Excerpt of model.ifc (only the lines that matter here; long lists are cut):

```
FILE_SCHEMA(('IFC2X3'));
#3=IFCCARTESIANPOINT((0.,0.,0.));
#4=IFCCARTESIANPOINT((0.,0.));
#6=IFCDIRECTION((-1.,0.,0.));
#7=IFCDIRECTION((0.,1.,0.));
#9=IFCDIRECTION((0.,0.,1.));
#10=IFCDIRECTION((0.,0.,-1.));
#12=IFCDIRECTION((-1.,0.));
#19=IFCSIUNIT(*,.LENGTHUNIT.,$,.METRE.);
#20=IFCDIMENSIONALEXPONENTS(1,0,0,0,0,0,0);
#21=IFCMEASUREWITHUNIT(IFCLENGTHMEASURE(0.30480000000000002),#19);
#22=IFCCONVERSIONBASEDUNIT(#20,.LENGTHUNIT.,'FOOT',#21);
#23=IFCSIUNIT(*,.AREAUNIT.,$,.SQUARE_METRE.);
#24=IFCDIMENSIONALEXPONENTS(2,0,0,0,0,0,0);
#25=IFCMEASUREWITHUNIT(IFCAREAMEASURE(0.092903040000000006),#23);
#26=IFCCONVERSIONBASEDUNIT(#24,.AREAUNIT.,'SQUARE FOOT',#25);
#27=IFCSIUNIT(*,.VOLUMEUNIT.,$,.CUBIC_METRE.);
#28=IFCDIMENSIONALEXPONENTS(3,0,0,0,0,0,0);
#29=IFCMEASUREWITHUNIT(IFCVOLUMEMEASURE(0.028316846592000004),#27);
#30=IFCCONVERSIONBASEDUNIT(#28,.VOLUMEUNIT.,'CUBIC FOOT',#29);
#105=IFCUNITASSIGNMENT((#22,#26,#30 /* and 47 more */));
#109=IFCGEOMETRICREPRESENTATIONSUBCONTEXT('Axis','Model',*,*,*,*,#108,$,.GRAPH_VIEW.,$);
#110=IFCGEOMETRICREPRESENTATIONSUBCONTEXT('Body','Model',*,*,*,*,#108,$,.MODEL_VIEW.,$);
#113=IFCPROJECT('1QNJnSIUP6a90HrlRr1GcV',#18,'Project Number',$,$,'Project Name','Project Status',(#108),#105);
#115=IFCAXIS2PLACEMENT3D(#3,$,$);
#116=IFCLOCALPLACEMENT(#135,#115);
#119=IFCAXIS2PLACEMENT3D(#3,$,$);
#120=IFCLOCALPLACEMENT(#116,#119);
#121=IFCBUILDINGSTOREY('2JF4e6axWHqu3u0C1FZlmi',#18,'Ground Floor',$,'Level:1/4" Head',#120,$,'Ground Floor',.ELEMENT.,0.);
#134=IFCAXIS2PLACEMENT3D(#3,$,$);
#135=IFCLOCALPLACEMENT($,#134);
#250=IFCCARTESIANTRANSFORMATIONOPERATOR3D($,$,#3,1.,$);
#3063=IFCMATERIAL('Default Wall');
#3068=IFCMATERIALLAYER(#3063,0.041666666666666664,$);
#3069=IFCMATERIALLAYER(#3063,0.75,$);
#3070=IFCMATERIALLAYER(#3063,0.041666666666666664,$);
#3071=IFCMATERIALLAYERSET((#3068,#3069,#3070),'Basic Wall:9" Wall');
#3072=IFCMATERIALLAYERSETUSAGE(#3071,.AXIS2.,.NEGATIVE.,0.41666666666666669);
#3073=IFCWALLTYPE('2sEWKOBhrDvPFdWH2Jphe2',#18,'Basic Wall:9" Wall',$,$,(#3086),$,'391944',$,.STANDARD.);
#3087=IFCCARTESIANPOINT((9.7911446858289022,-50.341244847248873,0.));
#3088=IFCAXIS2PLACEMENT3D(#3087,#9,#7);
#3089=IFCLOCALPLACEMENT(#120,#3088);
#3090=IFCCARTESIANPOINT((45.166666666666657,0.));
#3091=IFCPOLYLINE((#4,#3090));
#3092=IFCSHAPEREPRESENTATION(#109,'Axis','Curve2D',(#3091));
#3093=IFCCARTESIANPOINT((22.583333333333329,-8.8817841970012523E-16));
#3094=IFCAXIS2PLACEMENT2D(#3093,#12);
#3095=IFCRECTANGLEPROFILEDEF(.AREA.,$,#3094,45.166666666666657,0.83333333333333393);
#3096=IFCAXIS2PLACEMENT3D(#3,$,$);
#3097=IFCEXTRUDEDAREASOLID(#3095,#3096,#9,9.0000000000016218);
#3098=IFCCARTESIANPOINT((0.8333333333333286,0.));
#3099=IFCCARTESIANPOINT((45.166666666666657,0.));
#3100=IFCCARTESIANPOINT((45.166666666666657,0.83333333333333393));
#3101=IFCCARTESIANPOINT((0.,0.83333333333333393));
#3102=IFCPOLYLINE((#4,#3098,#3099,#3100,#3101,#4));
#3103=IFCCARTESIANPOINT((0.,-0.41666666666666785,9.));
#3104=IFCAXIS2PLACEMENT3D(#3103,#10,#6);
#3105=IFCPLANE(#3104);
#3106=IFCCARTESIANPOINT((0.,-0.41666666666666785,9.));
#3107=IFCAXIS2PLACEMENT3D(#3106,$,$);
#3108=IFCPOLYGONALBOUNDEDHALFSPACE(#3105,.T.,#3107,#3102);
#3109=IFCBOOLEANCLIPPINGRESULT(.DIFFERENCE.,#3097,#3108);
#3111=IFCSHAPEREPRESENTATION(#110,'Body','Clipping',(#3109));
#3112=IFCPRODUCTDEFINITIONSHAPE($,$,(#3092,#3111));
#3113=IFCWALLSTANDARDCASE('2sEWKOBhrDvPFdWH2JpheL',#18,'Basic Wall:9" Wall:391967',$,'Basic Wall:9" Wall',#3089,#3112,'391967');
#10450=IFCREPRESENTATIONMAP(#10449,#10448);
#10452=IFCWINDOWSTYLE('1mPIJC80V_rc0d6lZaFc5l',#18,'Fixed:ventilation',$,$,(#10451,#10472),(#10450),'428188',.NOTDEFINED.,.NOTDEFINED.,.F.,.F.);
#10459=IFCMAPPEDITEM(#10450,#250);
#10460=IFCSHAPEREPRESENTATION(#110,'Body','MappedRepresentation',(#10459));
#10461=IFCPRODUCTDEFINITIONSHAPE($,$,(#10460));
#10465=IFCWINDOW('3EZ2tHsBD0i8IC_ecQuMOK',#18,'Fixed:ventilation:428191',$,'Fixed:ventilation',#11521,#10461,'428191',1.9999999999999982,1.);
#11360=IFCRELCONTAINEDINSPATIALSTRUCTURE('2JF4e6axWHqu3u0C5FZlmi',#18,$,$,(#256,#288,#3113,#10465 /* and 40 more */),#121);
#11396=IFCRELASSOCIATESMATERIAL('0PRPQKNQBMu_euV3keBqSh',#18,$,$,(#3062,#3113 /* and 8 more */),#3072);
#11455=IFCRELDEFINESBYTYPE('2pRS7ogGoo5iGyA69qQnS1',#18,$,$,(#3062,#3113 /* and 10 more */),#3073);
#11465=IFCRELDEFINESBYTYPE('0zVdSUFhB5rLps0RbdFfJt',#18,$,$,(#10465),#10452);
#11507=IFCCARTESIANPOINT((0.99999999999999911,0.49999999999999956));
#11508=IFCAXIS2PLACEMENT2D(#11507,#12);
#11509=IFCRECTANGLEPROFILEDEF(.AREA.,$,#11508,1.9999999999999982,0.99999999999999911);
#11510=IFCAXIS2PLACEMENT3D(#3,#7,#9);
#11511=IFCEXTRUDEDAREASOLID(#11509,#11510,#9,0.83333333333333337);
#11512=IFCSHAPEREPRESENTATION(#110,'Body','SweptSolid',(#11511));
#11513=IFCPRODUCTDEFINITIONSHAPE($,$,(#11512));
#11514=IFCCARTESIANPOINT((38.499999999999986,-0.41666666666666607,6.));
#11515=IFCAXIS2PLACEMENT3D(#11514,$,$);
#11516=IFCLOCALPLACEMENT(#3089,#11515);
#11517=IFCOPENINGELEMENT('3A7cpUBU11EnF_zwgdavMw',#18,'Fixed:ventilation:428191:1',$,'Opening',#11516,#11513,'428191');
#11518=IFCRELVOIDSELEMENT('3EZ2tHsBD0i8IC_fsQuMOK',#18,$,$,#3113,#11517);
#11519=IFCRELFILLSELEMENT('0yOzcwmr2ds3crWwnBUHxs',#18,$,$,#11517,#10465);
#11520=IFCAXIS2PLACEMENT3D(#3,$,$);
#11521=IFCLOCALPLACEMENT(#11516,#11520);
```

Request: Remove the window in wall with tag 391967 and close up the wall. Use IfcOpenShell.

```python
import ifcopenshell
import ifcopenshell.api.feature
import ifcopenshell.api.root
import ifcopenshell.geom
import ifcopenshell.util.shape

model = ifcopenshell.open("model.ifc")
settings = ifcopenshell.geom.settings()


def volume(element):
    """Net volume in cubic metres, openings subtracted."""
    shape = ifcopenshell.geom.create_shape(settings, element)
    return ifcopenshell.util.shape.get_volume(shape.geometry)


window = model.by_id(10465)
opening = window.FillsVoids[0].RelatingOpeningElement
wall = opening.VoidsElements[0].RelatingBuildingElement
before = volume(wall)

ifcopenshell.api.root.remove_product(model, product=window)
ifcopenshell.api.feature.remove_feature(model, feature=opening)

after = volume(wall)

print(f"wall volume {before:.3f} -> {after:.3f} m3")

model.write("model-out.ifc")
```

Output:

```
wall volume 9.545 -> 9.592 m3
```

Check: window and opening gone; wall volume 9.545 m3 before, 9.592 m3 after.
